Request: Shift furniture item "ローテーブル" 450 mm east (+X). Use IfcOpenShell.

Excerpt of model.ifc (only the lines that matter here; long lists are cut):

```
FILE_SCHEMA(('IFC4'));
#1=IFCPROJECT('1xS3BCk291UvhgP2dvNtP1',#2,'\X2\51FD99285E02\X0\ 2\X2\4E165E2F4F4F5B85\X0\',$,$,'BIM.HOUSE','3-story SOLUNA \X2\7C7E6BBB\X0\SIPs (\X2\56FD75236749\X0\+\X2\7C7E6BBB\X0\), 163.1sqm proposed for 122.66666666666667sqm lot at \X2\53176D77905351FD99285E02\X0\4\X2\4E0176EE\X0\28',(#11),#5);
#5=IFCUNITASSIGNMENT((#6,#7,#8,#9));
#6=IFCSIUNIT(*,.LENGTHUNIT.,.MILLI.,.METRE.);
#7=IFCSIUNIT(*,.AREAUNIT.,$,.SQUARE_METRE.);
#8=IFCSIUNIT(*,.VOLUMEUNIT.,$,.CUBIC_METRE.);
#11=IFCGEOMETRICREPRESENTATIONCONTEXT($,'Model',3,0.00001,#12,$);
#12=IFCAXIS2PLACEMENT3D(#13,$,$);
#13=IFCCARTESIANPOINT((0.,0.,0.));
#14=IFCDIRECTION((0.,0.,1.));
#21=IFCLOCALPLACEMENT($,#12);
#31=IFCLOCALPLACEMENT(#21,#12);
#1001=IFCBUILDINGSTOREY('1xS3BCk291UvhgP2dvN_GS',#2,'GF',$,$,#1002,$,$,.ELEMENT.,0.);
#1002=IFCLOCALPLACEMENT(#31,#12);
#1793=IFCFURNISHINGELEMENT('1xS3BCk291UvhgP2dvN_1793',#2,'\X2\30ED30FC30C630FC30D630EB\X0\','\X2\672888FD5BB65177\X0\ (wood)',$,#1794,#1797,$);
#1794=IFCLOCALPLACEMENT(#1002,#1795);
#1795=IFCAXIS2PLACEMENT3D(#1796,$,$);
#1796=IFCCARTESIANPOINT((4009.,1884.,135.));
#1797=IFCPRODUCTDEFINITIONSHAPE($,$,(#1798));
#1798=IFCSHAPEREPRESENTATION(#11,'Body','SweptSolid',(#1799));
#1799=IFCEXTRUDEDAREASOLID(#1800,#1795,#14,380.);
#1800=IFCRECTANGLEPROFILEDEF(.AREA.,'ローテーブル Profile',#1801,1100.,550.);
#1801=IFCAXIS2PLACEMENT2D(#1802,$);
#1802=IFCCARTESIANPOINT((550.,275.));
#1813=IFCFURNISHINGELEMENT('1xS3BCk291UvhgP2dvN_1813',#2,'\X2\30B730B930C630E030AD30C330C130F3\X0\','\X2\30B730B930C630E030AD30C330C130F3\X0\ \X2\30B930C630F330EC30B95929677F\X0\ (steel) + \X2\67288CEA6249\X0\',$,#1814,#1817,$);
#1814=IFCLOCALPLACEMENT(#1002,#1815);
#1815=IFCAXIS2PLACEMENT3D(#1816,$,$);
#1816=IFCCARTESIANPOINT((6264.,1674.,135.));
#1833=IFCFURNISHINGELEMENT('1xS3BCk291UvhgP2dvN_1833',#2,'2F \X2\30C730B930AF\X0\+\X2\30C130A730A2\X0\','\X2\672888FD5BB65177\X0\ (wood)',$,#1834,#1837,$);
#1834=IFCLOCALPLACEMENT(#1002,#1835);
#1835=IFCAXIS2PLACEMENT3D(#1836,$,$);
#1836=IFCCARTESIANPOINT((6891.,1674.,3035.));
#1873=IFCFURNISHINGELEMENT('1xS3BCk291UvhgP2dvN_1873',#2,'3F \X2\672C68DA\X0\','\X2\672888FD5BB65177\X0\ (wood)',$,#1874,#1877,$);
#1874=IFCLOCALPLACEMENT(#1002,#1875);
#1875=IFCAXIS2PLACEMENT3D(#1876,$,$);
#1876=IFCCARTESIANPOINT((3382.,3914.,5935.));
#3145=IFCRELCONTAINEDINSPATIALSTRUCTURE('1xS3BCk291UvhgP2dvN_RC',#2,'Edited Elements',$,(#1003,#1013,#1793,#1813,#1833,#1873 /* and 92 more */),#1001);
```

```python
import ifcopenshell
import ifcopenshell.api.geometry
import ifcopenshell.util.placement
import ifcopenshell.util.unit

model = ifcopenshell.open("model.ifc")
unit_scale = ifcopenshell.util.unit.calculate_unit_scale(model)

item = model.by_guid("1xS3BCk291UvhgP2dvN_1793")
matrix = ifcopenshell.util.placement.get_local_placement(item.ObjectPlacement)
matrix[0, 3] += 0.45 / unit_scale
ifcopenshell.api.geometry.edit_object_placement(model, product=item, matrix=matrix, is_si=False)

print(ifcopenshell.util.placement.get_local_placement(item.ObjectPlacement).round(3) + 0.0)

model.write("model_v2.ifc")
```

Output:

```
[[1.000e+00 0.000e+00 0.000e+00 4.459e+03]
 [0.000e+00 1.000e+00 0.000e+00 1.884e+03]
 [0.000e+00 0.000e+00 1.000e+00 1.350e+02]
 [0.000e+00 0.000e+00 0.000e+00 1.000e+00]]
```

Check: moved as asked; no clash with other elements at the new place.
